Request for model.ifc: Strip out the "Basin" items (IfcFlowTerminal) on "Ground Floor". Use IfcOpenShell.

First a look at what the model holds.

```python
import ifcopenshell
import ifcopenshell.util.element

model = ifcopenshell.open("model.ifc")
print(model.schema)
storey = next(s for s in model.by_type("IfcBuildingStorey") if s.Name == "Ground Floor")
terminals = [e for e in ifcopenshell.util.element.get_decomposition(storey) if e.is_a("IfcFlowTerminal")]
seen = {}
for e in terminals:
    element_type = ifcopenshell.util.element.get_type(e)
    name = element_type.Name if element_type not in (None, e) else None
    seen[name] = seen.get(name, 0) + 1
for name, count in sorted(seen.items(), key=str):
    print(count, "x", name)
```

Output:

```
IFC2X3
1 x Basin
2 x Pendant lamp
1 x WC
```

```python
import ifcopenshell
import ifcopenshell.api.root
import ifcopenshell.util.element

model = ifcopenshell.open("model.ifc")

storey = next(s for s in model.by_type("IfcBuildingStorey") if s.Name == "Ground Floor")
terminals = [e for e in ifcopenshell.util.element.get_decomposition(storey) if e.is_a("IfcFlowTerminal")]
targets = [e for e in terminals if (t := ifcopenshell.util.element.get_type(e)) not in (None, e) and t.Name == "Basin"]

for e in targets:
    ifcopenshell.api.root.remove_product(model, product=e)
print(len(targets), "removed")

model.write("model_updated.ifc")
```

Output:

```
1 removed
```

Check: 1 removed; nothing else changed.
